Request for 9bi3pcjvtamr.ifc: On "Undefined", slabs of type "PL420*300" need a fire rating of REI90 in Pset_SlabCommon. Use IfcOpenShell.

First a look at what the model holds.

```python
import ifcopenshell
import ifcopenshell.util.element

model = ifcopenshell.open("9bi3pcjvtamr.ifc")
print(model.schema)
storey = next(s for s in model.by_type("IfcBuildingStorey") if s.Name == "Undefined")
slabs = [e for e in ifcopenshell.util.element.get_decomposition(storey) if e.is_a("IfcSlab")]
seen = {}
for e in slabs:
    element_type = ifcopenshell.util.element.get_type(e)
    key = (element_type.Name if element_type != e and element_type else None, ifcopenshell.util.element.get_pset(e, "Pset_SlabCommon", "FireRating"))
    seen[key] = seen.get(key, 0) + 1
for (name, value), count in sorted(seen.items(), key=str):
    print(count, "x", name, "|", value)
```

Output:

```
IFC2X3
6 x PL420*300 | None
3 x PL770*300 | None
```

```python
import ifcopenshell
import ifcopenshell.api.pset
import ifcopenshell.util.element

model = ifcopenshell.open("9bi3pcjvtamr.ifc")

storey = next(s for s in model.by_type("IfcBuildingStorey") if s.Name == "Undefined")
slabs = [e for e in ifcopenshell.util.element.get_decomposition(storey) if e.is_a("IfcSlab")]

count = 0
for e in slabs:
    element_type = ifcopenshell.util.element.get_type(e)
    if element_type in (None, e) or element_type.Name != "PL420*300":
        continue
    found = ifcopenshell.util.element.get_pset(e, "Pset_SlabCommon", should_inherit=False)
    if found:
        pset = model.by_id(found["id"])
        if len(ifcopenshell.util.element.get_elements_by_pset(pset)) > 1:
            pset = ifcopenshell.api.pset.unshare_pset(model, products=[e], pset=pset)[0]
    else:
        pset = ifcopenshell.api.pset.add_pset(model, product=e, name="Pset_SlabCommon")
    ifcopenshell.api.pset.edit_pset(model, pset=pset, properties={"FireRating": "REI90"})
    count += 1

print(count, "slabs updated")

model.write("9bi3pcjvtamr_v2.ifc")
```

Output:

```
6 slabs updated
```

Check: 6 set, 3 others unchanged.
